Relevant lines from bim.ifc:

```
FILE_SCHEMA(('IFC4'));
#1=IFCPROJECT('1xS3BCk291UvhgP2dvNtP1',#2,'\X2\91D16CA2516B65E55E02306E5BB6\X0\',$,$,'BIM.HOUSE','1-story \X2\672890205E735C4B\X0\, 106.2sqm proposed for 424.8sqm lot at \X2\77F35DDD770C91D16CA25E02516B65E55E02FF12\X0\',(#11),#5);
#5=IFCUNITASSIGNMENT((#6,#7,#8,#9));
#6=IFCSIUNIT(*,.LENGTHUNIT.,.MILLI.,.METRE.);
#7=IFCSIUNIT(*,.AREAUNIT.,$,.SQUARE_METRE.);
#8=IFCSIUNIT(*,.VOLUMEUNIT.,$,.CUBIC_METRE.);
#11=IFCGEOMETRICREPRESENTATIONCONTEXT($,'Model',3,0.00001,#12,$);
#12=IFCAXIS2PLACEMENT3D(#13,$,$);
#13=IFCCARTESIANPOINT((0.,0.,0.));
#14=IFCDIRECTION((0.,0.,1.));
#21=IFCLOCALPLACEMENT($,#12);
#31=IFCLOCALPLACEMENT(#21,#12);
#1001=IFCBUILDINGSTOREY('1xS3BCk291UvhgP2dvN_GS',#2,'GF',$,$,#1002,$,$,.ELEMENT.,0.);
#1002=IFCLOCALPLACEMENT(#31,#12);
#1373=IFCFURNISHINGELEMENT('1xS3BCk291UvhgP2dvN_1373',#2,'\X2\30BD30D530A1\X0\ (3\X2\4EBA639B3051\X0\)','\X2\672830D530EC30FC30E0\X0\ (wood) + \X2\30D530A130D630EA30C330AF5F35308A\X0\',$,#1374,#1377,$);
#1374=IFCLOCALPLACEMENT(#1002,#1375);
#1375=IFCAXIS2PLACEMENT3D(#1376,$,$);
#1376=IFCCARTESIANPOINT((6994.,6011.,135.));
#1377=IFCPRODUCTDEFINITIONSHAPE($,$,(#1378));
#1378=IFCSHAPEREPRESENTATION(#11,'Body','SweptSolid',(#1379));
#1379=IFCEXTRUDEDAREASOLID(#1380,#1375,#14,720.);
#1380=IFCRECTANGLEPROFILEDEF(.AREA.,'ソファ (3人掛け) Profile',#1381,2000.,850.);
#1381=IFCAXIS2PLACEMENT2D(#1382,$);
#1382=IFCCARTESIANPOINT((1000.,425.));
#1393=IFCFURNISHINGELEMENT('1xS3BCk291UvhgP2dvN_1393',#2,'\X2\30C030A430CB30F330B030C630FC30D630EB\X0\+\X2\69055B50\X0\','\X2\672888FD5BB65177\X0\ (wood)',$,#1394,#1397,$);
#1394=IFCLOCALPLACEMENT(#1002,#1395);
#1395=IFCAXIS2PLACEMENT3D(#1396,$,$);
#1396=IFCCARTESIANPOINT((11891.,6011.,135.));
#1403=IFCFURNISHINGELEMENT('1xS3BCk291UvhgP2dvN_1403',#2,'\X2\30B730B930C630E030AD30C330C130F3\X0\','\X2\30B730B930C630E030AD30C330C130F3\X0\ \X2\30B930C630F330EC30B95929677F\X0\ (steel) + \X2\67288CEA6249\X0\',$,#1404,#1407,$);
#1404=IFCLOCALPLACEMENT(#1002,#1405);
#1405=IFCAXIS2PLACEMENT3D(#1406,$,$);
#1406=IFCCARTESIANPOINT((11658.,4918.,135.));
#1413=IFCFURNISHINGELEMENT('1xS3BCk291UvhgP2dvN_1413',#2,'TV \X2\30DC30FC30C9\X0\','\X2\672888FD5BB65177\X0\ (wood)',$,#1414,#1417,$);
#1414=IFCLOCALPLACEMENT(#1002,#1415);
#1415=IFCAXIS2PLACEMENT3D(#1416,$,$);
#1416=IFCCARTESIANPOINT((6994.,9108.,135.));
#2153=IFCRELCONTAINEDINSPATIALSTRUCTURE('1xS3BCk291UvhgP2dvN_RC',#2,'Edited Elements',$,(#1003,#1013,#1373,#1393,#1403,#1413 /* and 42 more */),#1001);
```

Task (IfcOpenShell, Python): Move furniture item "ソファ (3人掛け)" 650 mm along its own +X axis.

```python
import ifcopenshell
import ifcopenshell.api.geometry
import ifcopenshell.util.placement
import ifcopenshell.util.unit

model = ifcopenshell.open("bim.ifc")
unit_scale = ifcopenshell.util.unit.calculate_unit_scale(model)

item = model.by_id(1373)
matrix = ifcopenshell.util.placement.get_local_placement(item.ObjectPlacement)
matrix[:3, 3] += matrix[:3, 0] * 0.65 / unit_scale
ifcopenshell.api.geometry.edit_object_placement(model, product=item, matrix=matrix, is_si=False)

print(ifcopenshell.util.placement.get_local_placement(item.ObjectPlacement).round(3) + 0.0)

model.write("bim_rev.ifc")
```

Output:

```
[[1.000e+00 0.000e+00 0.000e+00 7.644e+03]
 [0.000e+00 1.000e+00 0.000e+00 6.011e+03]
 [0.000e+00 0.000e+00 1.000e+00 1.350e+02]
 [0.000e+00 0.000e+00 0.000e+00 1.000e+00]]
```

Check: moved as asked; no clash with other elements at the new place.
